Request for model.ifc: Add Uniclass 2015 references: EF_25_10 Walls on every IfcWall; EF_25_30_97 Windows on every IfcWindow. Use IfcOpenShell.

First a look at what the model holds.

```python
import ifcopenshell

model = ifcopenshell.open("model.ifc")
print(model.schema)
print("classifications:", [c.Name for c in model.by_type("IfcClassification")])
for ifc_class in ("IfcDoor", "IfcRoof", "IfcStair", "IfcWall", "IfcWindow"):
    print(ifc_class, len(model.by_type(ifc_class)))
```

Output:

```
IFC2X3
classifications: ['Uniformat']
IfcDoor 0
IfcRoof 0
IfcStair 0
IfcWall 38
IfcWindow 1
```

```python
import ifcopenshell
import ifcopenshell.api.classification

model = ifcopenshell.open("model.ifc")

# IFC2X3 requires Source and Edition and has no link from the project to the system.
system = model.create_entity("IfcClassification", Source="NBS", Edition="2015", Name="Uniclass 2015")

codes = {
    "IfcWall": ("EF_25_10", "Walls"),
    "IfcWindow": ("EF_25_30_97", "Windows"),
}
for ifc_class, (code, name) in codes.items():
    products = model.by_type(ifc_class)
    ifcopenshell.api.classification.add_reference(
        model, products=products, classification=system, identification=code, name=name
    )
    print(code, len(products))

model.write("model_edited.ifc")
```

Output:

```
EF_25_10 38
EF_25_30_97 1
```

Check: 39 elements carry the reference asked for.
